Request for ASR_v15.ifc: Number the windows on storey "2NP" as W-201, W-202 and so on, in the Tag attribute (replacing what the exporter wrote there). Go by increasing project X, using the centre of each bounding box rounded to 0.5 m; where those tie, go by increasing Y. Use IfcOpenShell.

First a look at what the model holds.

```python
import ifcopenshell
import ifcopenshell.util.element
import ifcopenshell.util.placement

model = ifcopenshell.open("ASR_v15.ifc")
print(model.schema)
storey = next(s for s in model.by_type("IfcBuildingStorey") if s.Name == "2NP")
windows = [e for e in ifcopenshell.util.element.get_decomposition(storey) if e.is_a("IfcWindow")]
for e in sorted(windows, key=lambda e: e.id()):
    origin = ifcopenshell.util.placement.get_local_placement(e.ObjectPlacement)[:3, 3]
    print(e.id(), e.Tag, e.Name, origin.round(2) + 0.0, sep=" | ")
```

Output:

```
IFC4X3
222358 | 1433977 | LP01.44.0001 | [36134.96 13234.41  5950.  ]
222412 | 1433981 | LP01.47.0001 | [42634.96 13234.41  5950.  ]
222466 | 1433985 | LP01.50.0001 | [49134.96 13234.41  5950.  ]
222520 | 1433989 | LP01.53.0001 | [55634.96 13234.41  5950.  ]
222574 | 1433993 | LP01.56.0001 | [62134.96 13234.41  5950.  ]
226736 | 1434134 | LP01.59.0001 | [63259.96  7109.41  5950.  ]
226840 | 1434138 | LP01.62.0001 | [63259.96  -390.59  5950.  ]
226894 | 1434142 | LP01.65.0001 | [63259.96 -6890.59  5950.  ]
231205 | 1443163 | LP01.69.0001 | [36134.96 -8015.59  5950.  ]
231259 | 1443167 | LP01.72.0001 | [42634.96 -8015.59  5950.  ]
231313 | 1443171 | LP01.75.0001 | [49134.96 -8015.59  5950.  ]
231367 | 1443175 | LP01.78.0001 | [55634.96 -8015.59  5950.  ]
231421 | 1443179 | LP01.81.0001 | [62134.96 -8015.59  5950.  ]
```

```python
import ifcopenshell
import ifcopenshell.geom
import ifcopenshell.util.element
import ifcopenshell.util.shape

model = ifcopenshell.open("ASR_v15.ifc")
settings = ifcopenshell.geom.settings()
settings.set("use-world-coords", True)


def centre(element):
    shape = ifcopenshell.geom.create_shape(settings, element)
    return ifcopenshell.util.shape.get_bbox_centroid(shape.geometry)


storey = next(s for s in model.by_type("IfcBuildingStorey") if s.Name == "2NP")
windows = [e for e in ifcopenshell.util.element.get_decomposition(storey) if e.is_a("IfcWindow")]

# Insertion points can sit at a corner or the storey origin, so sort by the geometry (in metres).
centres = {e: centre(e) for e in windows}
windows.sort(key=lambda e: (round(centres[e][0] / 0.5), centres[e][1]))

for i, e in enumerate(windows, start=1):
    number = f"W-2{i:02d}"
    e.Tag = number
    print(e.id(), number)

model.write("ASR_v15_rev.ifc")
```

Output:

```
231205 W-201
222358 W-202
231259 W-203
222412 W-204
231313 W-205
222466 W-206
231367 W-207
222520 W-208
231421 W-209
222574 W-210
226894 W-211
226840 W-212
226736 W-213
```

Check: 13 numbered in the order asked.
